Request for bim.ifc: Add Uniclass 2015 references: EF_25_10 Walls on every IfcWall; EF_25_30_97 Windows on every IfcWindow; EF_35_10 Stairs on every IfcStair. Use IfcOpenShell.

First a look at what the model holds.

```python
import ifcopenshell

model = ifcopenshell.open("bim.ifc")
print(model.schema)
print("classifications:", [c.Name for c in model.by_type("IfcClassification")])
for ifc_class in ("IfcDoor", "IfcRoof", "IfcStair", "IfcWall", "IfcWindow"):
    print(ifc_class, len(model.by_type(ifc_class)))
```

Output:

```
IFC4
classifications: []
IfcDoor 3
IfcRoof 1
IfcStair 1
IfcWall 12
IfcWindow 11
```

```python
import ifcopenshell
import ifcopenshell.api.classification

model = ifcopenshell.open("bim.ifc")

system = ifcopenshell.api.classification.add_classification(model, classification="Uniclass 2015")

codes = {
    "IfcWall": ("EF_25_10", "Walls"),
    "IfcWindow": ("EF_25_30_97", "Windows"),
    "IfcStair": ("EF_35_10", "Stairs"),
}
for ifc_class, (code, name) in codes.items():
    products = model.by_type(ifc_class)
    ifcopenshell.api.classification.add_reference(
        model, products=products, classification=system, identification=code, name=name
    )
    print(code, len(products))

model.write("bim_updated.ifc")
```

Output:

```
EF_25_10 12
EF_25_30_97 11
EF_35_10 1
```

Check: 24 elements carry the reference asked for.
